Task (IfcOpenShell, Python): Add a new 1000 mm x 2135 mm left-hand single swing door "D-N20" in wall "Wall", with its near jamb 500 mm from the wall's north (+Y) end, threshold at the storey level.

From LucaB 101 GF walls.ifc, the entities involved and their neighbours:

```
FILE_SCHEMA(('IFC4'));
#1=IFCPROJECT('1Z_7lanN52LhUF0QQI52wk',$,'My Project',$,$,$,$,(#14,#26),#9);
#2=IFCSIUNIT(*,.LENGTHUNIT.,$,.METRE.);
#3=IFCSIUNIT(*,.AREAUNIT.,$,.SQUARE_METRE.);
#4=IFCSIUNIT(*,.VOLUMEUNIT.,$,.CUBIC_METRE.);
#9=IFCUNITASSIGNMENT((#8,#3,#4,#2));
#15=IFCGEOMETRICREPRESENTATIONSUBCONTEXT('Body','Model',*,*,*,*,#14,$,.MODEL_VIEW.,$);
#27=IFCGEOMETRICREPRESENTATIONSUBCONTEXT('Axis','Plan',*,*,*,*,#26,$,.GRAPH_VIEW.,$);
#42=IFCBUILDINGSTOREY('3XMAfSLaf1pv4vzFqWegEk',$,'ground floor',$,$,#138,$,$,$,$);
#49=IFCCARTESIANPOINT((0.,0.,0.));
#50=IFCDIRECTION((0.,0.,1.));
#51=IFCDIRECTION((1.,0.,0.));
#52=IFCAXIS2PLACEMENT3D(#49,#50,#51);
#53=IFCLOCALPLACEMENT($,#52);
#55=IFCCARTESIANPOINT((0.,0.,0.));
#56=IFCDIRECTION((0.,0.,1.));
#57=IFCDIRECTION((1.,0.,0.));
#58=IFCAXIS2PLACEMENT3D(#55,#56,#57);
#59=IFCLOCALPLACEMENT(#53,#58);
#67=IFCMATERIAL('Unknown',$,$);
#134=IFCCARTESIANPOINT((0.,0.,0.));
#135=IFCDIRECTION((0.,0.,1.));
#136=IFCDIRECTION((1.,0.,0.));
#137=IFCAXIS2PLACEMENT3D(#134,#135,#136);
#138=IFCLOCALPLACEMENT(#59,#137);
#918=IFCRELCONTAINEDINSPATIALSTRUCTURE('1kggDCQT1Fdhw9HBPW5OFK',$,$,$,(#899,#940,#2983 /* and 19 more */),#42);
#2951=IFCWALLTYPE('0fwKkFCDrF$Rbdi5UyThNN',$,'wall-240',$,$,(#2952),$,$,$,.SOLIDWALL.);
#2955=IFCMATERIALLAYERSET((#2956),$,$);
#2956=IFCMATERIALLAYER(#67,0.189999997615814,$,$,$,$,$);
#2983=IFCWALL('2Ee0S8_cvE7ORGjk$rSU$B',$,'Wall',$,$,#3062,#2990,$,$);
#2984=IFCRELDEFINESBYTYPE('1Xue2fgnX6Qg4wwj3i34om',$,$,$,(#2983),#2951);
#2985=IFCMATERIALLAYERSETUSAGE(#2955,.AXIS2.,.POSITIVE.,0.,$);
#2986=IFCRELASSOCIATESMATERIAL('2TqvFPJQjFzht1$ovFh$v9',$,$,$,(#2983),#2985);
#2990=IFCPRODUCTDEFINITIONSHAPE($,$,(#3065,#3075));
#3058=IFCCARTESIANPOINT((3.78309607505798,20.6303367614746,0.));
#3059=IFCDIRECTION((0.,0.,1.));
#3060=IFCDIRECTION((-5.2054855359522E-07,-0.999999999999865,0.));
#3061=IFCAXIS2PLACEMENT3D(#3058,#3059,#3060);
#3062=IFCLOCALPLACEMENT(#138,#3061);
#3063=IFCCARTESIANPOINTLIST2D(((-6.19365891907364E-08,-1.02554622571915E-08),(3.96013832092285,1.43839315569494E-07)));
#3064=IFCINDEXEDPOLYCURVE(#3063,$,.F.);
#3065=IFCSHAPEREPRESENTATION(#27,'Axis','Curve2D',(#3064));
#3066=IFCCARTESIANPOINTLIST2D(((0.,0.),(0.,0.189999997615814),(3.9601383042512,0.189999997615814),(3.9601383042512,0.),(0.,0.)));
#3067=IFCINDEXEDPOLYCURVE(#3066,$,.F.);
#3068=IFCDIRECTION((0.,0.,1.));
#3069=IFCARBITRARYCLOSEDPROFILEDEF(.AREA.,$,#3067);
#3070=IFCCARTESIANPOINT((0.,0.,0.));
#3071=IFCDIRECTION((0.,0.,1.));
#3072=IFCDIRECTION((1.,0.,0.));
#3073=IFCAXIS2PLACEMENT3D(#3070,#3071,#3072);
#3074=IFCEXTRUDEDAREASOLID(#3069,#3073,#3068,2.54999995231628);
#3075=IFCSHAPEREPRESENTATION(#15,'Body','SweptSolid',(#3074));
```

```python
import numpy as np
import ifcopenshell
import ifcopenshell.api.feature
import ifcopenshell.api.geometry
import ifcopenshell.api.root
import ifcopenshell.api.spatial
import ifcopenshell.geom
import ifcopenshell.util.element
import ifcopenshell.util.placement
import ifcopenshell.util.representation
import ifcopenshell.util.shape
import ifcopenshell.util.unit

model = ifcopenshell.open("LucaB 101 GF walls.ifc")
unit_scale = ifcopenshell.util.unit.calculate_unit_scale(model)
settings = ifcopenshell.geom.settings()


def volume(element):
    """Net volume in cubic metres, openings subtracted."""
    shape = ifcopenshell.geom.create_shape(settings, element)
    return ifcopenshell.util.shape.get_volume(shape.geometry)


wall = model.by_guid("2Ee0S8_cvE7ORGjk$rSU$B")
storey = ifcopenshell.util.element.get_container(wall, ifc_class="IfcBuildingStorey")
context = ifcopenshell.util.representation.get_context(model, "Model", "Body", "MODEL_VIEW")
before = volume(wall)

width, height, from_end, sill = 1, 2.135, 0.5, 0.0  # metres

# The wall runs along its own X axis, and the end named is its -X end.
wall_shape = ifcopenshell.geom.create_shape(settings, wall)
x, y, z = ifcopenshell.util.shape.get_vertices(wall_shape.geometry).T
start = x.min() + from_end
face, thickness = float(y.min()), float(y.max() - y.min())
wall_matrix = ifcopenshell.util.placement.get_local_placement(wall.ObjectPlacement)
level = ifcopenshell.util.placement.get_local_placement(storey.ObjectPlacement)[2, 3]


def in_wall(x, y):
    """Placement at x, y metres in the wall's axes, at sill height."""
    matrix = wall_matrix.copy()
    matrix[:, 3] = wall_matrix @ np.array([x / unit_scale, y / unit_scale, 0.0, 1.0])
    matrix[2, 3] = level + sill / unit_scale
    return matrix


# Opening: a box that overshoots both wall faces by 50 mm.
opening = ifcopenshell.api.root.create_entity(model, ifc_class="IfcOpeningElement", predefined_type="OPENING")
box = ifcopenshell.api.geometry.add_wall_representation(
    model, context=context, length=width, height=height, thickness=thickness + 0.1
)
ifcopenshell.api.geometry.assign_representation(model, product=opening, representation=box)
ifcopenshell.api.geometry.edit_object_placement(model, product=opening, matrix=in_wall(start, face - 0.05), is_si=False)
ifcopenshell.api.feature.add_feature(model, feature=opening, element=wall)

door = ifcopenshell.api.root.create_entity(model, ifc_class="IfcDoor", name="D-N20", predefined_type="DOOR")
door.OverallWidth, door.OverallHeight = width / unit_scale, height / unit_scale
door.OperationType = "SINGLE_SWING_LEFT"
body = ifcopenshell.api.geometry.add_door_representation(
    model,
    context=context,
    overall_width=door.OverallWidth,
    overall_height=door.OverallHeight,
    operation_type="SINGLE_SWING_LEFT",
    lining_properties={"LiningDepth": thickness / unit_scale, "ThresholdDepth": thickness / unit_scale},
)
ifcopenshell.api.geometry.assign_representation(model, product=door, representation=body)
ifcopenshell.api.spatial.assign_container(model, products=[door], relating_structure=storey)
ifcopenshell.api.feature.add_filling(model, opening=opening, element=door)

# The lining spans the wall, so the door starts at the wall face.
ifcopenshell.api.geometry.edit_object_placement(model, product=door, matrix=in_wall(start, face), is_si=False)

after = volume(wall)

print(f"wall volume {before:.3f} -> {after:.3f} m3")

model.write("LucaB 101 GF walls_rev.ifc")
```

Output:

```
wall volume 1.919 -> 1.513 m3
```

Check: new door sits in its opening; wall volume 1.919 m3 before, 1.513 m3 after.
